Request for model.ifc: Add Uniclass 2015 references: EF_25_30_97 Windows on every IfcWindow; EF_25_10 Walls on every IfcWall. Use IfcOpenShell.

First a look at what the model holds.

```python
import ifcopenshell

model = ifcopenshell.open("model.ifc")
print(model.schema)
print("classifications:", [c.Name for c in model.by_type("IfcClassification")])
for ifc_class in ("IfcDoor", "IfcRoof", "IfcStair", "IfcWall", "IfcWindow"):
    print(ifc_class, len(model.by_type(ifc_class)))
```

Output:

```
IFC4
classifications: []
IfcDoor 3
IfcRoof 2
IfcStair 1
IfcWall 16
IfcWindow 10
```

```python
import ifcopenshell
import ifcopenshell.api.classification

model = ifcopenshell.open("model.ifc")

system = ifcopenshell.api.classification.add_classification(model, classification="Uniclass 2015")

codes = {
    "IfcWindow": ("EF_25_30_97", "Windows"),
    "IfcWall": ("EF_25_10", "Walls"),
}
for ifc_class, (code, name) in codes.items():
    products = model.by_type(ifc_class)
    ifcopenshell.api.classification.add_reference(
        model, products=products, classification=system, identification=code, name=name
    )
    print(code, len(products))

model.write("model_edited.ifc")
```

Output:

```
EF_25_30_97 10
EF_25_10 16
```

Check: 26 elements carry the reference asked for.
